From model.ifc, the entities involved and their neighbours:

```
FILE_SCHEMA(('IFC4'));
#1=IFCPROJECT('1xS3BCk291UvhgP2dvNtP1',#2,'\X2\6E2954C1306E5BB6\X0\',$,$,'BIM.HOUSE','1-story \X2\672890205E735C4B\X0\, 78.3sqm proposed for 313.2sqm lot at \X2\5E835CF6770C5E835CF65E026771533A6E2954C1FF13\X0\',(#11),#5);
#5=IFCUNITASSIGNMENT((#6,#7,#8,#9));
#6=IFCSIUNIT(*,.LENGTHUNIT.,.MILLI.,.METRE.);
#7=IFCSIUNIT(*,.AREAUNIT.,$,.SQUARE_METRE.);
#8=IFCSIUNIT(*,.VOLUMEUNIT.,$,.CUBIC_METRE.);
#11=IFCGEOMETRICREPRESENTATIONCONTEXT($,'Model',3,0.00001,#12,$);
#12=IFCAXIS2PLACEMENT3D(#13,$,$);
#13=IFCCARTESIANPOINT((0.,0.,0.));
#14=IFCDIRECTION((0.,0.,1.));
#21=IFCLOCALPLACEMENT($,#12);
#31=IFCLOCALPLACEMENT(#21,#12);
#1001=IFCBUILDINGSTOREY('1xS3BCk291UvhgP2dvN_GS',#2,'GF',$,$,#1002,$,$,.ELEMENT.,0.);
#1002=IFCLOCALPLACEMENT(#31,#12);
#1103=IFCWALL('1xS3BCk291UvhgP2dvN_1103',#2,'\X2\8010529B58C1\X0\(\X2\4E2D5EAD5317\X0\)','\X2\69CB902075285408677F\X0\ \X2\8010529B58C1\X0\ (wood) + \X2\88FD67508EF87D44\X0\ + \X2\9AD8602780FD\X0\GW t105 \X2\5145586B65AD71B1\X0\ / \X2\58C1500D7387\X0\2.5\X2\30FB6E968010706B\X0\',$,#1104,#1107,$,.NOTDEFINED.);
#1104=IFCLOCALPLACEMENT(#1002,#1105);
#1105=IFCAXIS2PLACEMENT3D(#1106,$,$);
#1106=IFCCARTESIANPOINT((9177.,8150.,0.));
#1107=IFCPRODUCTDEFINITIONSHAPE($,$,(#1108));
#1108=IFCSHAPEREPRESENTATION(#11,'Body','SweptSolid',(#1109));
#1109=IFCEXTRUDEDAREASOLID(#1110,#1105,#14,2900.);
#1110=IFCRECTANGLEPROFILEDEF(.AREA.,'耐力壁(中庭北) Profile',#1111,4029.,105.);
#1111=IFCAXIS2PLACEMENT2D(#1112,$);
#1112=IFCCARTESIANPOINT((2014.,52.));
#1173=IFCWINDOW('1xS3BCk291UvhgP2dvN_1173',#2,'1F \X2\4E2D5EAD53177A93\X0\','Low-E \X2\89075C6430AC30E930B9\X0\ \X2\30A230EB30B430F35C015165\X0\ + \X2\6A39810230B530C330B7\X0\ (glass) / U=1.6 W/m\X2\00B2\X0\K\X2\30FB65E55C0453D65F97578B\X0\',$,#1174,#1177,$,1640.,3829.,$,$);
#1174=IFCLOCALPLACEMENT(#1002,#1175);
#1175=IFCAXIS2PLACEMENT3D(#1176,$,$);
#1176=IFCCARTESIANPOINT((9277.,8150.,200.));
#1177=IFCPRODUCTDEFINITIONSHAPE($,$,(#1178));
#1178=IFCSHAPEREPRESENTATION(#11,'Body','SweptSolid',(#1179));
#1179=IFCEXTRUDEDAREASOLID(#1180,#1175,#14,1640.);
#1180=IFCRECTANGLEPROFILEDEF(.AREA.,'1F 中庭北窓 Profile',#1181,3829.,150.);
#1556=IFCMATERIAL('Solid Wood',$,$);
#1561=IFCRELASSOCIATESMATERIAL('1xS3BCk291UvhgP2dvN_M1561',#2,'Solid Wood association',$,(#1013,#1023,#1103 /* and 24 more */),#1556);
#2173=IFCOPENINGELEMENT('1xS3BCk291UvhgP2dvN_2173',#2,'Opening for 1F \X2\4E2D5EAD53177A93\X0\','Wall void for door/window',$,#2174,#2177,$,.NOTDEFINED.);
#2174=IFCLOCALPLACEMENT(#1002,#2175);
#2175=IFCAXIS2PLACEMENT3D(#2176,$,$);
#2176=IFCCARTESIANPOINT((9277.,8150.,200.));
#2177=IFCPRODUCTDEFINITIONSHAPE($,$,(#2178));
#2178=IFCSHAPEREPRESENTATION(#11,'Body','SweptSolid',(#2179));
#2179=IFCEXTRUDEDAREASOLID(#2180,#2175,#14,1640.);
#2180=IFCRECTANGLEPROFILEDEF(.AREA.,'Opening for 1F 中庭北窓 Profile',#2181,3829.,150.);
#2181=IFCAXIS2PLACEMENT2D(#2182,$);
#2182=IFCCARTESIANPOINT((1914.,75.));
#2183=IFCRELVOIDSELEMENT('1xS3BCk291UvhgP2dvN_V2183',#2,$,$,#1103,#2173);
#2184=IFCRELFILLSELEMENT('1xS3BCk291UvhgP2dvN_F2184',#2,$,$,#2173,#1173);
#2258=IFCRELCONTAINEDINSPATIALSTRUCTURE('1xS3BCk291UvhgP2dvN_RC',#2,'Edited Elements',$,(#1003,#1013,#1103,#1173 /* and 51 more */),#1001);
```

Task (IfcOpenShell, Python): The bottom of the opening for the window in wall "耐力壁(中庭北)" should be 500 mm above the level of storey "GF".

```python
import numpy as np
import ifcopenshell
import ifcopenshell.api.geometry
import ifcopenshell.geom
import ifcopenshell.util.element
import ifcopenshell.util.placement
import ifcopenshell.util.shape
import ifcopenshell.util.unit

model = ifcopenshell.open("model.ifc")
unit_scale = ifcopenshell.util.unit.calculate_unit_scale(model)

window = model.by_id(1173)
opening = window.FillsVoids[0].RelatingOpeningElement
storey = ifcopenshell.util.element.get_container(window, ifc_class="IfcBuildingStorey")
level = ifcopenshell.util.placement.get_local_placement(storey.ObjectPlacement)[2, 3]

# The opening's origin need not be at the sill, so measure its lowest point.
shape = ifcopenshell.geom.create_shape(ifcopenshell.geom.settings(), opening)
bottom = ifcopenshell.util.shape.get_shape_bottom_elevation(shape, shape.geometry) / unit_scale
dz = level + 0.5 / unit_scale - bottom

shift = np.array([0.0, 0.0, dz])
# The window is not placed relative to its opening, so move both.
for product in (opening, window):
    matrix = ifcopenshell.util.placement.get_local_placement(product.ObjectPlacement)
    matrix[:3, 3] += shift
    ifcopenshell.api.geometry.edit_object_placement(model, product=product, matrix=matrix, is_si=False)

print(f"moved by {dz * unit_scale:+.3f} m")

model.write("model-out.ifc")
```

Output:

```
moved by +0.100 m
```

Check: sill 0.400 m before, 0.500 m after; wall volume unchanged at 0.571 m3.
